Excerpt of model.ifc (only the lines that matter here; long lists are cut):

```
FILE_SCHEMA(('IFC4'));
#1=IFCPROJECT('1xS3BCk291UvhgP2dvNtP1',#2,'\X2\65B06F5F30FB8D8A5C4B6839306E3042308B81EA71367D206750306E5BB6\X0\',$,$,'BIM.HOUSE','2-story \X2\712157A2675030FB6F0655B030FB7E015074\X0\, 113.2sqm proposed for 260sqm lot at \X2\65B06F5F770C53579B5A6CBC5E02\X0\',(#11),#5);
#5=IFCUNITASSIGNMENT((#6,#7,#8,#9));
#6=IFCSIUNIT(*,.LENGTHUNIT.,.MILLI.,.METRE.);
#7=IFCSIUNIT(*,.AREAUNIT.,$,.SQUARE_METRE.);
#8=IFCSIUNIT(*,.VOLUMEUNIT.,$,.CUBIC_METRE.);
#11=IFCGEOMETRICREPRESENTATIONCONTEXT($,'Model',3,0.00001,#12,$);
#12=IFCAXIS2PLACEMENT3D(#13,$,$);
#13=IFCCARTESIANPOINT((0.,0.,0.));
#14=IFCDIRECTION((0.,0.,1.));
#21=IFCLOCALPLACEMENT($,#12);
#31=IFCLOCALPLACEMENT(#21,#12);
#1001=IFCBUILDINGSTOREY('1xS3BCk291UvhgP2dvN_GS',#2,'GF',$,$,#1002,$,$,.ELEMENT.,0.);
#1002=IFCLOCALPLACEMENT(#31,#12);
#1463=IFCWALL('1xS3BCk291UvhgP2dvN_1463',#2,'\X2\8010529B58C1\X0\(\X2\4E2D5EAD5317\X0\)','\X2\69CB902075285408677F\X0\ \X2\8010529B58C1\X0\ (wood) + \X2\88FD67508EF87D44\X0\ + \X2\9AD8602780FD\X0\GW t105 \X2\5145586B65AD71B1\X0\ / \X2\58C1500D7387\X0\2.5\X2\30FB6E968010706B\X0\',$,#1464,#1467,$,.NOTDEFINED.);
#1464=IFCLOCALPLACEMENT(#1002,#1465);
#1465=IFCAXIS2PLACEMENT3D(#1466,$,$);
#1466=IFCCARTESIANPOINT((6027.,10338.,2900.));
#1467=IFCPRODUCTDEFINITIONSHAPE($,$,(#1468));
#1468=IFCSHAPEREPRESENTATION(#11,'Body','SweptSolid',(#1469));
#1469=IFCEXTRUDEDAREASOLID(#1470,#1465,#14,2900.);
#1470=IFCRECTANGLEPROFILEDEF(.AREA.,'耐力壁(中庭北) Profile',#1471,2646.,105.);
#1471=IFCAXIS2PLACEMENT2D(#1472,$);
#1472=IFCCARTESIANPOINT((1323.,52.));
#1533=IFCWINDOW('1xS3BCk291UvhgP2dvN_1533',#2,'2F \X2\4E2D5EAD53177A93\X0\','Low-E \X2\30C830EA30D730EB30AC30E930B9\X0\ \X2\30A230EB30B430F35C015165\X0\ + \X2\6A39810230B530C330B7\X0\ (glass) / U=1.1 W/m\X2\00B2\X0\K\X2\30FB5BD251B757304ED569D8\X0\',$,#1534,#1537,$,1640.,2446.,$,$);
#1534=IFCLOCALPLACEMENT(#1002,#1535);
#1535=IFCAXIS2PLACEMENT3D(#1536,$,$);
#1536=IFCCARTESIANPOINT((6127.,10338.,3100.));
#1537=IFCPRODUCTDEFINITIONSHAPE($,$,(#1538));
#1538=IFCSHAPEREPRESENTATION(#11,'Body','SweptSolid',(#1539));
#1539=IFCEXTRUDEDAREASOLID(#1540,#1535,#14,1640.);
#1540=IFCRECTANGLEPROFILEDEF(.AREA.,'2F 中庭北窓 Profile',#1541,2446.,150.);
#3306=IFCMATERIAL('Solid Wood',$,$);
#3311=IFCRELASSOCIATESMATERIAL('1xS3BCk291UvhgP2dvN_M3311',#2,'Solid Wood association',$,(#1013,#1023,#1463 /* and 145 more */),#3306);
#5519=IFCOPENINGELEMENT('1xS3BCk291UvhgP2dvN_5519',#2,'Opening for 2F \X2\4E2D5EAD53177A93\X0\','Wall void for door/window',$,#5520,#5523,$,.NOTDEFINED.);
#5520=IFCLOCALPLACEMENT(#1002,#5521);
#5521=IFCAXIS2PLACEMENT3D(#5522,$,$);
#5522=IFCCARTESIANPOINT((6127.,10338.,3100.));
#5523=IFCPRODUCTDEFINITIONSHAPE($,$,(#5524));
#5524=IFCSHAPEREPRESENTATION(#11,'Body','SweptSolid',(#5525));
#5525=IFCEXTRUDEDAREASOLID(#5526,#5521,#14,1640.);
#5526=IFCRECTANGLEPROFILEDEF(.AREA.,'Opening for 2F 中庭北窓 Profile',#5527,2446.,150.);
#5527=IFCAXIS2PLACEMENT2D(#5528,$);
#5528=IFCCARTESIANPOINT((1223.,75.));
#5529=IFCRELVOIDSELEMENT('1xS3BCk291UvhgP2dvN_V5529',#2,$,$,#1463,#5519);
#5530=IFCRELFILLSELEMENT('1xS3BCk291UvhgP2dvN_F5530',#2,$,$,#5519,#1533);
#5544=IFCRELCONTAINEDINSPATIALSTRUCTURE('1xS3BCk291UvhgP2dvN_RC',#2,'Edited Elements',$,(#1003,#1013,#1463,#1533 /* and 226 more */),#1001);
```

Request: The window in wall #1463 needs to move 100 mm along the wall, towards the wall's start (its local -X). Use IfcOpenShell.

```python
import ifcopenshell
import ifcopenshell.api.geometry
import ifcopenshell.util.placement
import ifcopenshell.util.unit

model = ifcopenshell.open("model.ifc")
unit_scale = ifcopenshell.util.unit.calculate_unit_scale(model)

window = model.by_guid("1xS3BCk291UvhgP2dvN_1533")
opening = window.FillsVoids[0].RelatingOpeningElement
wall = opening.VoidsElements[0].RelatingBuildingElement

wall_matrix = ifcopenshell.util.placement.get_local_placement(wall.ObjectPlacement)
shift = wall_matrix[:3, 0] * -0.1 / unit_scale
before = ifcopenshell.util.placement.get_local_placement(window.ObjectPlacement)[:3, 3].copy()

# The window is not placed relative to its opening, so move both.
for product in (opening, window):
    matrix = ifcopenshell.util.placement.get_local_placement(product.ObjectPlacement)
    matrix[:3, 3] += shift
    ifcopenshell.api.geometry.edit_object_placement(model, product=product, matrix=matrix, is_si=False)

after = ifcopenshell.util.placement.get_local_placement(window.ObjectPlacement)[:3, 3]
print("window moved by", (after - before).round(3) + 0.0)

model.write("model_v2.ifc")
```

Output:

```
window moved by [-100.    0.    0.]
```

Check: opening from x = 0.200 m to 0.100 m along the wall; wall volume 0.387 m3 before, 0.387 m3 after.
